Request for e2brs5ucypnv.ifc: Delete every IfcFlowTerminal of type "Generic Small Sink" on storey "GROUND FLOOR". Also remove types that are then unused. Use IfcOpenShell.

First a look at what the model holds.

```python
import ifcopenshell
import ifcopenshell.util.element

model = ifcopenshell.open("e2brs5ucypnv.ifc")
print(model.schema)
storey = next(s for s in model.by_type("IfcBuildingStorey") if s.Name == "GROUND FLOOR")
terminals = [e for e in ifcopenshell.util.element.get_decomposition(storey) if e.is_a("IfcFlowTerminal")]
seen = {}
for e in terminals:
    element_type = ifcopenshell.util.element.get_type(e)
    name = element_type.Name if element_type not in (None, e) else None
    seen[name] = seen.get(name, 0) + 1
for name, count in sorted(seen.items(), key=str):
    print(count, "x", name)
```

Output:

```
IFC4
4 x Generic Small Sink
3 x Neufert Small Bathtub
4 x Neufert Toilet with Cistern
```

```python
import ifcopenshell
import ifcopenshell.api.root
import ifcopenshell.util.element

model = ifcopenshell.open("e2brs5ucypnv.ifc")

storey = next(s for s in model.by_type("IfcBuildingStorey") if s.Name == "GROUND FLOOR")
terminals = [e for e in ifcopenshell.util.element.get_decomposition(storey) if e.is_a("IfcFlowTerminal")]
targets = [e for e in terminals if (t := ifcopenshell.util.element.get_type(e)) not in (None, e) and t.Name == "Generic Small Sink"]
types = {ifcopenshell.util.element.get_type(e) for e in targets} - {None, *targets}

for e in targets:
    ifcopenshell.api.root.remove_product(model, product=e)
print(len(targets), "removed")

unused = [t for t in types if not ifcopenshell.util.element.get_types(t)]
for t in unused:
    ifcopenshell.api.root.remove_product(model, product=t)
print(len(unused), "unused types removed")

model.write("e2brs5ucypnv_updated.ifc")
```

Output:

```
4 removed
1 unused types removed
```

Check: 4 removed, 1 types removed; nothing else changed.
